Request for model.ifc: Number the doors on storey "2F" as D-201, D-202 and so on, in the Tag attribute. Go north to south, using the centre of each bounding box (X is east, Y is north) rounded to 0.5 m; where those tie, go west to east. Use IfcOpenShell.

First a look at what the model holds.

```python
import ifcopenshell
import ifcopenshell.util.element
import ifcopenshell.util.placement

model = ifcopenshell.open("model.ifc")
print(model.schema)
storey = next(s for s in model.by_type("IfcBuildingStorey") if s.Name == "2F")
doors = [e for e in ifcopenshell.util.element.get_decomposition(storey) if e.is_a("IfcDoor")]
for e in sorted(doors, key=lambda e: e.id()):
    origin = ifcopenshell.util.placement.get_local_placement(e.ObjectPlacement)[:3, 3]
    print(e.id(), e.Tag, e.Name, origin.round(2) + 0.0, sep=" | ")
```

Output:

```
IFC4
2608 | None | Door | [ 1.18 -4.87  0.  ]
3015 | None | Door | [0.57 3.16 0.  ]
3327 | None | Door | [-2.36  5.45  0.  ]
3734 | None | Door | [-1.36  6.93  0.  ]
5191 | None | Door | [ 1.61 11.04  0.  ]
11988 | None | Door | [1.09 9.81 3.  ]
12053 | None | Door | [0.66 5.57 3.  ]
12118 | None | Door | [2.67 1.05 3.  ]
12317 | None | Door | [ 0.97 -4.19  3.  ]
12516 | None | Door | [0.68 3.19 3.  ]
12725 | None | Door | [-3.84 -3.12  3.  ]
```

```python
import ifcopenshell
import ifcopenshell.geom
import ifcopenshell.util.element
import ifcopenshell.util.shape

model = ifcopenshell.open("model.ifc")
settings = ifcopenshell.geom.settings()
settings.set("use-world-coords", True)


def centre(element):
    shape = ifcopenshell.geom.create_shape(settings, element)
    return ifcopenshell.util.shape.get_bbox_centroid(shape.geometry)


storey = next(s for s in model.by_type("IfcBuildingStorey") if s.Name == "2F")
doors = [e for e in ifcopenshell.util.element.get_decomposition(storey) if e.is_a("IfcDoor")]

# Insertion points can sit at a corner or the storey origin, so sort by the geometry (in metres).
centres = {e: centre(e) for e in doors}
doors.sort(key=lambda e: (-round(centres[e][1] / 0.5), centres[e][0]))

for i, e in enumerate(doors, start=1):
    number = f"D-2{i:02d}"
    e.Tag = number
    print(e.id(), number)

model.write("model-out.ifc")
```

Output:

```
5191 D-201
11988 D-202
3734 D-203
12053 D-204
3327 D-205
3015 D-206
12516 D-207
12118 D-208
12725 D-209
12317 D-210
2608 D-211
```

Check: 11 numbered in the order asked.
